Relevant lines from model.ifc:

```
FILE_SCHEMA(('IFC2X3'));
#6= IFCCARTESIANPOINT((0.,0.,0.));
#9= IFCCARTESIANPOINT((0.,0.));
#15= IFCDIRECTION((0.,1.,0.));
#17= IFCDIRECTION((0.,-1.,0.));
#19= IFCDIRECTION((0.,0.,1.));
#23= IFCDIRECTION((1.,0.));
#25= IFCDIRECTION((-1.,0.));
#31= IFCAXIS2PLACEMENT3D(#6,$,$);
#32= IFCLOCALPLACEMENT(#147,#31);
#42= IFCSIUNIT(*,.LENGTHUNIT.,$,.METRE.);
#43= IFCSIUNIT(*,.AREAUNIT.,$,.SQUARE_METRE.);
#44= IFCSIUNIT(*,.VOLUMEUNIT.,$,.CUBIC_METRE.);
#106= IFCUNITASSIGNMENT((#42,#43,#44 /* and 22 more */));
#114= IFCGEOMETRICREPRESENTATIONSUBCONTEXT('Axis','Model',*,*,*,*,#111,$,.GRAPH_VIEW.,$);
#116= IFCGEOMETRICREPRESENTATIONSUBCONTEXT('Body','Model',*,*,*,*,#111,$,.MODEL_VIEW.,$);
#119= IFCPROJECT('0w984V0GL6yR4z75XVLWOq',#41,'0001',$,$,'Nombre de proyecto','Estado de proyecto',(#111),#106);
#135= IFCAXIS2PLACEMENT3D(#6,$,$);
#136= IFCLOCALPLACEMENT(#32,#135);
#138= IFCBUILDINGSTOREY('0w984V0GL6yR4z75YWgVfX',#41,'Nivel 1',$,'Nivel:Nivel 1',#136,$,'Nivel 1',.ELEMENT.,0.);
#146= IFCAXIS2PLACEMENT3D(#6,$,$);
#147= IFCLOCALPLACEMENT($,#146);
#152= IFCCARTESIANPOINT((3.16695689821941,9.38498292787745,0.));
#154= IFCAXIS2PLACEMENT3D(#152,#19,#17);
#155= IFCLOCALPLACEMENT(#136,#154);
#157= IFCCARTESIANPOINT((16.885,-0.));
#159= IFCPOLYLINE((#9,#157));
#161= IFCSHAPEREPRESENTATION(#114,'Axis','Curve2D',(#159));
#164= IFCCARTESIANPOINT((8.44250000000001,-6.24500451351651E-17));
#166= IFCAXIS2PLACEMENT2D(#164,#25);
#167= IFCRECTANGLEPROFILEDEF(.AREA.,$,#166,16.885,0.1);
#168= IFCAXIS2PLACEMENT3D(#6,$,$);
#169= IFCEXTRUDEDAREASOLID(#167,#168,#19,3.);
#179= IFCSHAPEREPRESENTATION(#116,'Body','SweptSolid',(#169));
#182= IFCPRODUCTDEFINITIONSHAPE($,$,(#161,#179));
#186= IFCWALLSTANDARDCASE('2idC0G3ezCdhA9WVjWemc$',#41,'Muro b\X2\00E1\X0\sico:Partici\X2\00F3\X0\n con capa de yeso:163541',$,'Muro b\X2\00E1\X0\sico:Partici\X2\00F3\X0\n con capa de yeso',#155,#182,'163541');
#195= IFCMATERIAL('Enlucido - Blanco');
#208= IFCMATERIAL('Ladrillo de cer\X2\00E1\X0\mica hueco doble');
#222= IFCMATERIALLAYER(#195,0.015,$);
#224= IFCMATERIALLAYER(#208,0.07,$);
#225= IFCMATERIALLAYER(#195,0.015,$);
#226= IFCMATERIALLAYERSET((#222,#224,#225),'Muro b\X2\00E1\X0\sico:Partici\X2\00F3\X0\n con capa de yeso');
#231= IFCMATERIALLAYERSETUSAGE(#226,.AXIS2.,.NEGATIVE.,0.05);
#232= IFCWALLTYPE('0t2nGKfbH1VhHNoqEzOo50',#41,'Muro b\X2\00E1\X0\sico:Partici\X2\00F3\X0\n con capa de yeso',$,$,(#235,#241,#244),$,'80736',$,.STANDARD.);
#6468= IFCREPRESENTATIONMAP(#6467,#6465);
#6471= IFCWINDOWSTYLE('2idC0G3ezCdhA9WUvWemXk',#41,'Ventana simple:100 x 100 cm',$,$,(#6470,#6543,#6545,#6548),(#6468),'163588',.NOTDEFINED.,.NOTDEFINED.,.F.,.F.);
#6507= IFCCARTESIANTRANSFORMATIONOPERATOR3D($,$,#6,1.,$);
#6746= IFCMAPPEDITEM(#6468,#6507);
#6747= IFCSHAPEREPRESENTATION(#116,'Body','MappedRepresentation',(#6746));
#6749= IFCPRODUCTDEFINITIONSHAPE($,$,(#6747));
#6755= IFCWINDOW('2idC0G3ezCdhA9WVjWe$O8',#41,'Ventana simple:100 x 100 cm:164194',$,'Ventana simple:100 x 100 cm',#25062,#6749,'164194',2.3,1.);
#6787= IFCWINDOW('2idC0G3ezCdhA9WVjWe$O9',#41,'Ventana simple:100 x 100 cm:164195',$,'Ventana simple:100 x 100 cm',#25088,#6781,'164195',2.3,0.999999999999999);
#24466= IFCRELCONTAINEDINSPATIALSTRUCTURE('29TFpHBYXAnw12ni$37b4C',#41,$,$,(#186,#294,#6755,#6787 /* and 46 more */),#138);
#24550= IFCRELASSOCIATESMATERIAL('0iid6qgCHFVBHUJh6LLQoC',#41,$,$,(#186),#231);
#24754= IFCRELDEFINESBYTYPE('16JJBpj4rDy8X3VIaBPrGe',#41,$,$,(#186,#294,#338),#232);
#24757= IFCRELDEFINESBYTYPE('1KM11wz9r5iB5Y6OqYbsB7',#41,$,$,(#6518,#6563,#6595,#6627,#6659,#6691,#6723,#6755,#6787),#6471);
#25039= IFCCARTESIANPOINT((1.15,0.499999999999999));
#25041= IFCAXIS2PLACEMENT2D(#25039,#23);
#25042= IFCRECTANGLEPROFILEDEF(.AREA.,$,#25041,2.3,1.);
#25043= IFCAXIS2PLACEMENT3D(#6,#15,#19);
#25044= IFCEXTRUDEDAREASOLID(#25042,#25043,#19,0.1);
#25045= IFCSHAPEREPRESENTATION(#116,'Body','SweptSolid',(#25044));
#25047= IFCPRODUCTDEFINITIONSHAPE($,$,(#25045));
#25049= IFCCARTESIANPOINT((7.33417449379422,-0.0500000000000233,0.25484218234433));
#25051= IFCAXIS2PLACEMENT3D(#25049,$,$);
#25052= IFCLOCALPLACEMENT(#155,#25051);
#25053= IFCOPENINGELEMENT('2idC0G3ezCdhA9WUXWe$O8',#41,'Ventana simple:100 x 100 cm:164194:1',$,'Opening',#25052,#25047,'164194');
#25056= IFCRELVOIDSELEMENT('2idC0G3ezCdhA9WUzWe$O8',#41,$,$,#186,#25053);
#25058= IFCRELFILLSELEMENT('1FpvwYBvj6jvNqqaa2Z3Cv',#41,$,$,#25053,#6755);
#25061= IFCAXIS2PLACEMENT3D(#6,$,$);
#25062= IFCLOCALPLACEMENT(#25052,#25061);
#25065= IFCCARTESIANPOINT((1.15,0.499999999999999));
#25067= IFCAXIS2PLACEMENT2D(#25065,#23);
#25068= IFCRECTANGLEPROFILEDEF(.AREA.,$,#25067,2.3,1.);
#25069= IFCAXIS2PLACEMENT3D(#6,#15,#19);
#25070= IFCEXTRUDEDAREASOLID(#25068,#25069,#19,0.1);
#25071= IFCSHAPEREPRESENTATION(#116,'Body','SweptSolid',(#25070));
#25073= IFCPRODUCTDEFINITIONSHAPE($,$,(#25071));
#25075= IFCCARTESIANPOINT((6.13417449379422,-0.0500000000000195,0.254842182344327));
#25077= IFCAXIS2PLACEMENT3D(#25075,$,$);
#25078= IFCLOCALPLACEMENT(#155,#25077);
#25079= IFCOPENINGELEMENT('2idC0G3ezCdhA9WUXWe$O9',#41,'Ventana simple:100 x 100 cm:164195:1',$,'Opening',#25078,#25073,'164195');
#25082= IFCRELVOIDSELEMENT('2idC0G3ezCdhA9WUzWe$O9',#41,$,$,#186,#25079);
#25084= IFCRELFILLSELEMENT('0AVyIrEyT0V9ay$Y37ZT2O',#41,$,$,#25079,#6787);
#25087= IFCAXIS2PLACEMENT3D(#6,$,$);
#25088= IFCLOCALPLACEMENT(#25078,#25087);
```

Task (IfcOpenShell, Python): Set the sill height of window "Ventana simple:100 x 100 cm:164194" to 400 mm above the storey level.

```python
import numpy as np
import ifcopenshell
import ifcopenshell.api.geometry
import ifcopenshell.geom
import ifcopenshell.util.element
import ifcopenshell.util.placement
import ifcopenshell.util.shape
import ifcopenshell.util.unit

model = ifcopenshell.open("model.ifc")
unit_scale = ifcopenshell.util.unit.calculate_unit_scale(model)

window = model.by_id(6755)
opening = window.FillsVoids[0].RelatingOpeningElement
storey = ifcopenshell.util.element.get_container(window, ifc_class="IfcBuildingStorey")
level = ifcopenshell.util.placement.get_local_placement(storey.ObjectPlacement)[2, 3]

# The opening's origin need not be at the sill, so measure its lowest point.
shape = ifcopenshell.geom.create_shape(ifcopenshell.geom.settings(), opening)
bottom = ifcopenshell.util.shape.get_shape_bottom_elevation(shape, shape.geometry) / unit_scale
dz = level + 0.4 / unit_scale - bottom

shift = np.array([0.0, 0.0, dz])
# The window is placed relative to its opening, so it follows when the opening moves.
matrix = ifcopenshell.util.placement.get_local_placement(opening.ObjectPlacement)
matrix[:3, 3] += shift
ifcopenshell.api.geometry.edit_object_placement(
    model, product=opening, matrix=matrix, is_si=False, should_transform_children=True
)

print(f"moved by {dz * unit_scale:+.3f} m")

model.write("model_v2.ifc")
```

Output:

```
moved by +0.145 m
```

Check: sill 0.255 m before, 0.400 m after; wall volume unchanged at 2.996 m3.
